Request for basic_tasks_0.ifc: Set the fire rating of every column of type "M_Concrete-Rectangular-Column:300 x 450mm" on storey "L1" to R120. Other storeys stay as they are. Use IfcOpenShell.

First a look at what the model holds.

```python
import ifcopenshell
import ifcopenshell.util.element

model = ifcopenshell.open("basic_tasks_0.ifc")
print(model.schema)
storey = next(s for s in model.by_type("IfcBuildingStorey") if s.Name == "L1")
columns = [e for e in ifcopenshell.util.element.get_decomposition(storey) if e.is_a("IfcColumn")]
seen = {}
for e in columns:
    element_type = ifcopenshell.util.element.get_type(e)
    key = (element_type.Name if element_type != e and element_type else None, ifcopenshell.util.element.get_pset(e, "Pset_ColumnCommon", "FireRating"))
    seen[key] = seen.get(key, 0) + 1
for (name, value), count in sorted(seen.items(), key=str):
    print(count, "x", name, "|", value)
```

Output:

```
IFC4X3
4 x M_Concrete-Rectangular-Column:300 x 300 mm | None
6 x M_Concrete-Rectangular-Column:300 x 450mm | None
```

```python
import ifcopenshell
import ifcopenshell.api.pset
import ifcopenshell.util.element

model = ifcopenshell.open("basic_tasks_0.ifc")

storey = next(s for s in model.by_type("IfcBuildingStorey") if s.Name == "L1")
columns = [e for e in ifcopenshell.util.element.get_decomposition(storey) if e.is_a("IfcColumn")]

count = 0
for e in columns:
    element_type = ifcopenshell.util.element.get_type(e)
    if element_type in (None, e) or element_type.Name != "M_Concrete-Rectangular-Column:300 x 450mm":
        continue
    # add_pset returns the element's existing set when there is one.
    pset = ifcopenshell.api.pset.add_pset(model, product=e, name="Pset_ColumnCommon")
    ifcopenshell.api.pset.edit_pset(model, pset=pset, properties={"FireRating": "R120"})
    count += 1

print(count, "columns updated")

model.write("basic_tasks_0-out.ifc")
```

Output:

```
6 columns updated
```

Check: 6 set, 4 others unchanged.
